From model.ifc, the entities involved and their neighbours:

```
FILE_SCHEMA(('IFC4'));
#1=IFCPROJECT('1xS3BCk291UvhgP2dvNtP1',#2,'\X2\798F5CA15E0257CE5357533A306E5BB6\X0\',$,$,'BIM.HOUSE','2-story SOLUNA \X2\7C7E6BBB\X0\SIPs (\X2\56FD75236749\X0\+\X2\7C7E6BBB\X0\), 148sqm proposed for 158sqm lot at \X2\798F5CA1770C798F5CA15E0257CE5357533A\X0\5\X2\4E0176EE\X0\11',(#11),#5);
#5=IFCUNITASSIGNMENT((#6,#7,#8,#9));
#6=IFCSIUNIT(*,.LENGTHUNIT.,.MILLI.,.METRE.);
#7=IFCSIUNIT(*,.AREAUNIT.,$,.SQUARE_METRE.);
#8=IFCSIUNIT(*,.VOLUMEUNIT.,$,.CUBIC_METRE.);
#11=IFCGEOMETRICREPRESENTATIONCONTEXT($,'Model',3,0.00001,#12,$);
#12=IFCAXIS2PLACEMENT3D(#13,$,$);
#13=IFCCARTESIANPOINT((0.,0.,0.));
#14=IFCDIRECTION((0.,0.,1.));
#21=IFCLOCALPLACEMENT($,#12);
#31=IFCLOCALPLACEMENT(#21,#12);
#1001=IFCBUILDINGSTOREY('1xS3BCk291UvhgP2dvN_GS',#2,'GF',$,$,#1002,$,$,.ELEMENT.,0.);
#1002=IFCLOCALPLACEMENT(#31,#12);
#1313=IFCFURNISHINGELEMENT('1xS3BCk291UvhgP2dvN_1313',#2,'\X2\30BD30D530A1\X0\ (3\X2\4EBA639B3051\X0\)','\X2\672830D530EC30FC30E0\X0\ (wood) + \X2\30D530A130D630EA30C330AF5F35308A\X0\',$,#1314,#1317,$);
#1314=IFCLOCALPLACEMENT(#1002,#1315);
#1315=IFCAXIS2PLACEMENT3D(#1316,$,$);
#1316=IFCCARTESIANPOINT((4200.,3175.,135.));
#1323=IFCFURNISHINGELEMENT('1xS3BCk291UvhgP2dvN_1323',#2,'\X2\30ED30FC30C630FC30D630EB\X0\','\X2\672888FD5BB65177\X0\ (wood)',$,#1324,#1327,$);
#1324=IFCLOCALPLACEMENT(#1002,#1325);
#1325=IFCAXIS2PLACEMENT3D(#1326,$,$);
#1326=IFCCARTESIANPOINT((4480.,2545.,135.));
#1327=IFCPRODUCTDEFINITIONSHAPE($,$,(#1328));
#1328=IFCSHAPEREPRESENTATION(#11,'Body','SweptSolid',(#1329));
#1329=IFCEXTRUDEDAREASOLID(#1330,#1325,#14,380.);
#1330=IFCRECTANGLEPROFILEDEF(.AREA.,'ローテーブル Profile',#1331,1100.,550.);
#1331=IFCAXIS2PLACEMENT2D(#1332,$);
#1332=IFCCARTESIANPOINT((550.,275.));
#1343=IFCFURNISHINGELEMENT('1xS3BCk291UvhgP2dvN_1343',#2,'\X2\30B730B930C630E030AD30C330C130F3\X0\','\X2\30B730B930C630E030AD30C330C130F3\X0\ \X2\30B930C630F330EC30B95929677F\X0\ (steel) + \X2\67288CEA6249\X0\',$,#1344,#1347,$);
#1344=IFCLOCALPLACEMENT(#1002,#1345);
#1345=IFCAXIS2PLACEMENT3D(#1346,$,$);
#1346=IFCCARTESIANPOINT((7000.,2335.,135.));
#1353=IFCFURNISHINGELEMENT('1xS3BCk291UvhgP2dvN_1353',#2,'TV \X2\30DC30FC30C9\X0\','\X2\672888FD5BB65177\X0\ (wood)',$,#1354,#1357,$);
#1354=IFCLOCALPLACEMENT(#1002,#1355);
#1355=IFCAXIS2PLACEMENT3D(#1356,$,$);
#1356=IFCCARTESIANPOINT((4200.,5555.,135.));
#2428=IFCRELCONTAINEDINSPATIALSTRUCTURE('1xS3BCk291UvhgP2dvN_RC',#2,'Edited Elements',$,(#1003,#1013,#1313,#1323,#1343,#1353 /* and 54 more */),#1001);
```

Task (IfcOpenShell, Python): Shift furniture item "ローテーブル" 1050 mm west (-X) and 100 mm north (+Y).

```python
import ifcopenshell
import ifcopenshell.api.geometry
import ifcopenshell.util.placement

model = ifcopenshell.open("model.ifc")

item = model.by_guid("1xS3BCk291UvhgP2dvN_1323")
matrix = ifcopenshell.util.placement.get_local_placement(item.ObjectPlacement)
matrix[0, 3] -= 1050.0
matrix[1, 3] += 100.0
ifcopenshell.api.geometry.edit_object_placement(model, product=item, matrix=matrix, is_si=False)

print(ifcopenshell.util.placement.get_local_placement(item.ObjectPlacement).round(3) + 0.0)

model.write("model_edited.ifc")
```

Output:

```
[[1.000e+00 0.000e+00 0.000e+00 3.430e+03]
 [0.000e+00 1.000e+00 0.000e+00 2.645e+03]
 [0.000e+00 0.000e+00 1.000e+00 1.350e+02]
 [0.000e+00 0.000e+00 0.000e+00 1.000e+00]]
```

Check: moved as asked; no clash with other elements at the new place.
